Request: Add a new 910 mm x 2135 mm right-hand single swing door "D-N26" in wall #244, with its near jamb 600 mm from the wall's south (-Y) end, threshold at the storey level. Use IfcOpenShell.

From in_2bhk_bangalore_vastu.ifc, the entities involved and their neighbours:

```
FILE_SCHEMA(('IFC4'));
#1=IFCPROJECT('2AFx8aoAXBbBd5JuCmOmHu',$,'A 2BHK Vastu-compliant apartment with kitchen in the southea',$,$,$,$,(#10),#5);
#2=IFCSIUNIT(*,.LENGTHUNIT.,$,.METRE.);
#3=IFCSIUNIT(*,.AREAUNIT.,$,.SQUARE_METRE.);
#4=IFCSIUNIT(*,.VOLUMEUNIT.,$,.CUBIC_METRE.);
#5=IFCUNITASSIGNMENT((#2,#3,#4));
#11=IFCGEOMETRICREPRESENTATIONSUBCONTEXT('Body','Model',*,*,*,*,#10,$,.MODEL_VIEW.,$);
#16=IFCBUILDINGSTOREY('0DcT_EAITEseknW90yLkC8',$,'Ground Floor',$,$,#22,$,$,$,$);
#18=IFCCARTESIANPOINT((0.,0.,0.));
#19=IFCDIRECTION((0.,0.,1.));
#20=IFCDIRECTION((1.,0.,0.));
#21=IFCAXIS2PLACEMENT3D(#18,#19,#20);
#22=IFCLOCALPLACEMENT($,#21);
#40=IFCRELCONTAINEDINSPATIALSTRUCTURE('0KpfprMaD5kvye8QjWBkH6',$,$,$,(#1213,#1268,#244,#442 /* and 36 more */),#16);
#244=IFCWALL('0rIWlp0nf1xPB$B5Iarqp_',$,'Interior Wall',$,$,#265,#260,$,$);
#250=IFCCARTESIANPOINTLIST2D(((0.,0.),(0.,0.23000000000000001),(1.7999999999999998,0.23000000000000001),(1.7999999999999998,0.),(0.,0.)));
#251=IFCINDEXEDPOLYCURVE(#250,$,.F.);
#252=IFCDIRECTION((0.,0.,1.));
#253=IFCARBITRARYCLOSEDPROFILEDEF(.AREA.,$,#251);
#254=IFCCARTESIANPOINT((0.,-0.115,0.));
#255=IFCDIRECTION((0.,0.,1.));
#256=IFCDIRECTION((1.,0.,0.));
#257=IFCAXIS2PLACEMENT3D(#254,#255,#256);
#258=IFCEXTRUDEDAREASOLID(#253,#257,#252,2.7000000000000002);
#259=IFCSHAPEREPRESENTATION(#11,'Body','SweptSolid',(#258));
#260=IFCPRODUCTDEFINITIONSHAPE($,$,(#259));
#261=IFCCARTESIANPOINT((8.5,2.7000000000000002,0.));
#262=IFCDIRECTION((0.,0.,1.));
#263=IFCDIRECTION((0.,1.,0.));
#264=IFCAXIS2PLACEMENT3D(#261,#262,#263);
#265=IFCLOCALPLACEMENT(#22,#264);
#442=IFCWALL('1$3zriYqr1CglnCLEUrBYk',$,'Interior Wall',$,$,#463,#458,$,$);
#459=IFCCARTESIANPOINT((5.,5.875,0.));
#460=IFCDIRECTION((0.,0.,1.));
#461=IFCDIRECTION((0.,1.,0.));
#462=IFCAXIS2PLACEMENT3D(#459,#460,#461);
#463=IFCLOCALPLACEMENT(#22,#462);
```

```python
import numpy as np
import ifcopenshell
import ifcopenshell.api.feature
import ifcopenshell.api.geometry
import ifcopenshell.api.root
import ifcopenshell.api.spatial
import ifcopenshell.geom
import ifcopenshell.util.element
import ifcopenshell.util.placement
import ifcopenshell.util.representation
import ifcopenshell.util.shape
import ifcopenshell.util.unit

model = ifcopenshell.open("in_2bhk_bangalore_vastu.ifc")
unit_scale = ifcopenshell.util.unit.calculate_unit_scale(model)
settings = ifcopenshell.geom.settings()


def volume(element):
    """Net volume in cubic metres, openings subtracted."""
    shape = ifcopenshell.geom.create_shape(settings, element)
    return ifcopenshell.util.shape.get_volume(shape.geometry)


wall = model.by_guid("0rIWlp0nf1xPB$B5Iarqp_")
storey = ifcopenshell.util.element.get_container(wall, ifc_class="IfcBuildingStorey")
context = ifcopenshell.util.representation.get_context(model, "Model", "Body", "MODEL_VIEW")
before = volume(wall)

width, height, from_end, sill = 0.91, 2.135, 0.6, 0.0  # metres

# The wall runs along its own X axis, and the end named is its -X end.
wall_shape = ifcopenshell.geom.create_shape(settings, wall)
x, y, z = ifcopenshell.util.shape.get_vertices(wall_shape.geometry).T
start = x.min() + from_end
face, thickness = float(y.min()), float(y.max() - y.min())
wall_matrix = ifcopenshell.util.placement.get_local_placement(wall.ObjectPlacement)
level = ifcopenshell.util.placement.get_local_placement(storey.ObjectPlacement)[2, 3]


def in_wall(x, y):
    """Placement at x, y metres in the wall's axes, at sill height."""
    matrix = wall_matrix.copy()
    matrix[:, 3] = wall_matrix @ np.array([x / unit_scale, y / unit_scale, 0.0, 1.0])
    matrix[2, 3] = level + sill / unit_scale
    return matrix


# Opening: a box that overshoots both wall faces by 50 mm.
opening = ifcopenshell.api.root.create_entity(model, ifc_class="IfcOpeningElement", predefined_type="OPENING")
box = ifcopenshell.api.geometry.add_wall_representation(
    model, context=context, length=width, height=height, thickness=thickness + 0.1
)
ifcopenshell.api.geometry.assign_representation(model, product=opening, representation=box)
ifcopenshell.api.geometry.edit_object_placement(model, product=opening, matrix=in_wall(start, face - 0.05), is_si=False)
ifcopenshell.api.feature.add_feature(model, feature=opening, element=wall)

door = ifcopenshell.api.root.create_entity(model, ifc_class="IfcDoor", name="D-N26", predefined_type="DOOR")
door.OverallWidth, door.OverallHeight = width / unit_scale, height / unit_scale
door.OperationType = "SINGLE_SWING_RIGHT"
body = ifcopenshell.api.geometry.add_door_representation(
    model,
    context=context,
    overall_width=door.OverallWidth,
    overall_height=door.OverallHeight,
    operation_type="SINGLE_SWING_RIGHT",
    lining_properties={"LiningDepth": thickness / unit_scale, "ThresholdDepth": thickness / unit_scale},
)
ifcopenshell.api.geometry.assign_representation(model, product=door, representation=body)
ifcopenshell.api.spatial.assign_container(model, products=[door], relating_structure=storey)
ifcopenshell.api.feature.add_filling(model, opening=opening, element=door)

# The lining spans the wall, so the door starts at the wall face.
ifcopenshell.api.geometry.edit_object_placement(model, product=door, matrix=in_wall(start, face), is_si=False)

after = volume(wall)

print(f"wall volume {before:.3f} -> {after:.3f} m3")

model.write("in_2bhk_bangalore_vastu_edited.ifc")
```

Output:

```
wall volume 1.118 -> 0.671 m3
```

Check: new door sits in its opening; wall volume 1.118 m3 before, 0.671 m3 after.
